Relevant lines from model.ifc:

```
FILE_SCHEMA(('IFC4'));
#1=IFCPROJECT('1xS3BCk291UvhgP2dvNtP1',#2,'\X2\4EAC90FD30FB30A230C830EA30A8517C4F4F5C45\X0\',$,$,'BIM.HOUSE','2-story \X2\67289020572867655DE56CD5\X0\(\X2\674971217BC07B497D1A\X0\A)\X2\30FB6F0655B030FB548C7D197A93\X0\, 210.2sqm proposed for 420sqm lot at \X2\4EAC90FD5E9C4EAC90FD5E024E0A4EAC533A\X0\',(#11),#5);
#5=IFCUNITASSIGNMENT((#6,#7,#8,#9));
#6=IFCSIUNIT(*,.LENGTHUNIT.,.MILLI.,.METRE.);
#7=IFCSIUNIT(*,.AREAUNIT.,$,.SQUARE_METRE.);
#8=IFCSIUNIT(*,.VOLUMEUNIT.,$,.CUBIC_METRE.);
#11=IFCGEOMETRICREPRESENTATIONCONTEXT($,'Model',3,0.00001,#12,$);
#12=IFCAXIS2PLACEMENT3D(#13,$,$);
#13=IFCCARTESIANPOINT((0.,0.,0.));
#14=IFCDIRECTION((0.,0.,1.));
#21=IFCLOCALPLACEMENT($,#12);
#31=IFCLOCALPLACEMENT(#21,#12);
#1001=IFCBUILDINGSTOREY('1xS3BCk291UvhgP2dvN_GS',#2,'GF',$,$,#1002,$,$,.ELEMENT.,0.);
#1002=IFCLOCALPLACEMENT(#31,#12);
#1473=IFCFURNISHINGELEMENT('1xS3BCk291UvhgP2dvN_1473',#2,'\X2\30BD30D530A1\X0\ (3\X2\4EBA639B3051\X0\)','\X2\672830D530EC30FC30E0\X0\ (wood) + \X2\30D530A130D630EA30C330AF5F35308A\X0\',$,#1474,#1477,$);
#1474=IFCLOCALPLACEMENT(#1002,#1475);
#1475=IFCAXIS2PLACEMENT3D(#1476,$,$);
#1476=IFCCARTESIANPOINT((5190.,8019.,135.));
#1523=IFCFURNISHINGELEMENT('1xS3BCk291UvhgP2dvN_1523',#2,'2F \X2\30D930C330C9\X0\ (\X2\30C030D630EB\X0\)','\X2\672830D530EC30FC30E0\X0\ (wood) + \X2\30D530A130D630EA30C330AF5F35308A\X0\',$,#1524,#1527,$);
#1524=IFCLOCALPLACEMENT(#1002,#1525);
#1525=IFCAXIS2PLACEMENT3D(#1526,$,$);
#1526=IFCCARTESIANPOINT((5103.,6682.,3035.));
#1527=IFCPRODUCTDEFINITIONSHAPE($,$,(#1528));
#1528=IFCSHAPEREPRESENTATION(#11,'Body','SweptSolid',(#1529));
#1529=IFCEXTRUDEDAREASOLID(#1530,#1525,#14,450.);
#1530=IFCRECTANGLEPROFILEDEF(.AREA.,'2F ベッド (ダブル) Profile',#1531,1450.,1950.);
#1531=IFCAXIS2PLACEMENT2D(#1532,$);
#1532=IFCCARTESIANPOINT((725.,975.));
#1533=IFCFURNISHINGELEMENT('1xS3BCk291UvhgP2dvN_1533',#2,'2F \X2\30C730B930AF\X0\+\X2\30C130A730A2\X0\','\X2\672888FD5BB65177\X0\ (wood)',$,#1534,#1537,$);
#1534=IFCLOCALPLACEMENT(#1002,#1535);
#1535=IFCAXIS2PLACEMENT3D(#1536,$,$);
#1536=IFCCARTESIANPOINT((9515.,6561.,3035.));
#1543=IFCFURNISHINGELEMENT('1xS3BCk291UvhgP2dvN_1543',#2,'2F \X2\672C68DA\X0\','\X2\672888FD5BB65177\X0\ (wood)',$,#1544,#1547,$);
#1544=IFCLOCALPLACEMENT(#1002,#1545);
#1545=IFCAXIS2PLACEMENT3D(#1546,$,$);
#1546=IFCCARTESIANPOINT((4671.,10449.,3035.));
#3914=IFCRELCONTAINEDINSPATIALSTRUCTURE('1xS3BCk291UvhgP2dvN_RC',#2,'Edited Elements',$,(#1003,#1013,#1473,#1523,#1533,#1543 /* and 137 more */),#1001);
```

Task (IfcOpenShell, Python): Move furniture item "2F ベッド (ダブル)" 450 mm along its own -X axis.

```python
import ifcopenshell
import ifcopenshell.api.geometry
import ifcopenshell.util.placement
import ifcopenshell.util.unit

model = ifcopenshell.open("model.ifc")
unit_scale = ifcopenshell.util.unit.calculate_unit_scale(model)

item = model.by_guid("1xS3BCk291UvhgP2dvN_1523")
matrix = ifcopenshell.util.placement.get_local_placement(item.ObjectPlacement)
matrix[:3, 3] -= matrix[:3, 0] * 0.45 / unit_scale
ifcopenshell.api.geometry.edit_object_placement(model, product=item, matrix=matrix, is_si=False)

print(ifcopenshell.util.placement.get_local_placement(item.ObjectPlacement).round(3) + 0.0)

model.write("model_v2.ifc")
```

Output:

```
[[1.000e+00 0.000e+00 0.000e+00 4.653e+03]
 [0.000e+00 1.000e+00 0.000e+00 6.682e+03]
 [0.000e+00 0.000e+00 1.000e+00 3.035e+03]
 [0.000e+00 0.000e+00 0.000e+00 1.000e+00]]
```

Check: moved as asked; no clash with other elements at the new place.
